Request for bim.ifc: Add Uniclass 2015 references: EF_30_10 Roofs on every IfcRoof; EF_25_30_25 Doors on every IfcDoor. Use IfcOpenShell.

First a look at what the model holds.

```python
import ifcopenshell

model = ifcopenshell.open("bim.ifc")
print(model.schema)
print("classifications:", [c.Name for c in model.by_type("IfcClassification")])
for ifc_class in ("IfcDoor", "IfcRoof", "IfcStair", "IfcWall", "IfcWindow"):
    print(ifc_class, len(model.by_type(ifc_class)))
```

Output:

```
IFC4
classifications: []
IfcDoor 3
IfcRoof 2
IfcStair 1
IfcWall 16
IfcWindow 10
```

```python
import ifcopenshell
import ifcopenshell.api.classification

model = ifcopenshell.open("bim.ifc")

system = ifcopenshell.api.classification.add_classification(model, classification="Uniclass 2015")

codes = {
    "IfcRoof": ("EF_30_10", "Roofs"),
    "IfcDoor": ("EF_25_30_25", "Doors"),
}
for ifc_class, (code, name) in codes.items():
    products = model.by_type(ifc_class)
    ifcopenshell.api.classification.add_reference(
        model, products=products, classification=system, identification=code, name=name
    )
    print(code, len(products))

model.write("bim_v2.ifc")
```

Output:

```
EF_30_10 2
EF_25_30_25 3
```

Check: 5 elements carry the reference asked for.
